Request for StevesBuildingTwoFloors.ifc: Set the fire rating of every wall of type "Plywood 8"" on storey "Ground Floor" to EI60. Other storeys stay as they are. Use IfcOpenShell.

First a look at what the model holds.

```python
import ifcopenshell
import ifcopenshell.util.element

model = ifcopenshell.open("StevesBuildingTwoFloors.ifc")
print(model.schema)
storey = next(s for s in model.by_type("IfcBuildingStorey") if s.Name == "Ground Floor")
walls = [e for e in ifcopenshell.util.element.get_decomposition(storey) if e.is_a("IfcWall")]
seen = {}
for e in walls:
    element_type = ifcopenshell.util.element.get_type(e)
    key = (element_type.Name if element_type != e and element_type else None, ifcopenshell.util.element.get_pset(e, "Pset_WallCommon", "FireRating"))
    seen[key] = seen.get(key, 0) + 1
for (name, value), count in sorted(seen.items(), key=str):
    print(count, "x", name, "|", value)
```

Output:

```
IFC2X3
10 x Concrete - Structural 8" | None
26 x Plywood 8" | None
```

```python
import ifcopenshell
import ifcopenshell.api.pset
import ifcopenshell.util.element

model = ifcopenshell.open("StevesBuildingTwoFloors.ifc")

storey = next(s for s in model.by_type("IfcBuildingStorey") if s.Name == "Ground Floor")
walls = [e for e in ifcopenshell.util.element.get_decomposition(storey) if e.is_a("IfcWall")]

count = 0
for e in walls:
    element_type = ifcopenshell.util.element.get_type(e)
    if element_type in (None, e) or element_type.Name != 'Plywood 8"':
        continue
    # add_pset returns the element's existing set when there is one.
    pset = ifcopenshell.api.pset.add_pset(model, product=e, name="Pset_WallCommon")
    ifcopenshell.api.pset.edit_pset(model, pset=pset, properties={"FireRating": "EI60"})
    count += 1

print(count, "walls updated")

model.write("StevesBuildingTwoFloors-out.ifc")
```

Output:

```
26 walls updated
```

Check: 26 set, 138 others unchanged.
